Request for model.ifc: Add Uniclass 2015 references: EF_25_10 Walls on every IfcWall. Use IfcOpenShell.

First a look at what the model holds.

```python
import ifcopenshell

model = ifcopenshell.open("model.ifc")
print(model.schema)
print("classifications:", [c.Name for c in model.by_type("IfcClassification")])
for ifc_class in ("IfcDoor", "IfcRoof", "IfcStair", "IfcWall", "IfcWindow"):
    print(ifc_class, len(model.by_type(ifc_class)))
```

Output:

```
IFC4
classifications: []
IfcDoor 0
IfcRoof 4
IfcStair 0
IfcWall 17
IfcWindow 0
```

```python
import ifcopenshell
import ifcopenshell.api.classification

model = ifcopenshell.open("model.ifc")

system = ifcopenshell.api.classification.add_classification(model, classification="Uniclass 2015")

codes = {
    "IfcWall": ("EF_25_10", "Walls"),
}
for ifc_class, (code, name) in codes.items():
    products = model.by_type(ifc_class)
    ifcopenshell.api.classification.add_reference(
        model, products=products, classification=system, identification=code, name=name
    )
    print(code, len(products))

model.write("model-out.ifc")
```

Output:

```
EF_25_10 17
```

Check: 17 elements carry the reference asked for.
